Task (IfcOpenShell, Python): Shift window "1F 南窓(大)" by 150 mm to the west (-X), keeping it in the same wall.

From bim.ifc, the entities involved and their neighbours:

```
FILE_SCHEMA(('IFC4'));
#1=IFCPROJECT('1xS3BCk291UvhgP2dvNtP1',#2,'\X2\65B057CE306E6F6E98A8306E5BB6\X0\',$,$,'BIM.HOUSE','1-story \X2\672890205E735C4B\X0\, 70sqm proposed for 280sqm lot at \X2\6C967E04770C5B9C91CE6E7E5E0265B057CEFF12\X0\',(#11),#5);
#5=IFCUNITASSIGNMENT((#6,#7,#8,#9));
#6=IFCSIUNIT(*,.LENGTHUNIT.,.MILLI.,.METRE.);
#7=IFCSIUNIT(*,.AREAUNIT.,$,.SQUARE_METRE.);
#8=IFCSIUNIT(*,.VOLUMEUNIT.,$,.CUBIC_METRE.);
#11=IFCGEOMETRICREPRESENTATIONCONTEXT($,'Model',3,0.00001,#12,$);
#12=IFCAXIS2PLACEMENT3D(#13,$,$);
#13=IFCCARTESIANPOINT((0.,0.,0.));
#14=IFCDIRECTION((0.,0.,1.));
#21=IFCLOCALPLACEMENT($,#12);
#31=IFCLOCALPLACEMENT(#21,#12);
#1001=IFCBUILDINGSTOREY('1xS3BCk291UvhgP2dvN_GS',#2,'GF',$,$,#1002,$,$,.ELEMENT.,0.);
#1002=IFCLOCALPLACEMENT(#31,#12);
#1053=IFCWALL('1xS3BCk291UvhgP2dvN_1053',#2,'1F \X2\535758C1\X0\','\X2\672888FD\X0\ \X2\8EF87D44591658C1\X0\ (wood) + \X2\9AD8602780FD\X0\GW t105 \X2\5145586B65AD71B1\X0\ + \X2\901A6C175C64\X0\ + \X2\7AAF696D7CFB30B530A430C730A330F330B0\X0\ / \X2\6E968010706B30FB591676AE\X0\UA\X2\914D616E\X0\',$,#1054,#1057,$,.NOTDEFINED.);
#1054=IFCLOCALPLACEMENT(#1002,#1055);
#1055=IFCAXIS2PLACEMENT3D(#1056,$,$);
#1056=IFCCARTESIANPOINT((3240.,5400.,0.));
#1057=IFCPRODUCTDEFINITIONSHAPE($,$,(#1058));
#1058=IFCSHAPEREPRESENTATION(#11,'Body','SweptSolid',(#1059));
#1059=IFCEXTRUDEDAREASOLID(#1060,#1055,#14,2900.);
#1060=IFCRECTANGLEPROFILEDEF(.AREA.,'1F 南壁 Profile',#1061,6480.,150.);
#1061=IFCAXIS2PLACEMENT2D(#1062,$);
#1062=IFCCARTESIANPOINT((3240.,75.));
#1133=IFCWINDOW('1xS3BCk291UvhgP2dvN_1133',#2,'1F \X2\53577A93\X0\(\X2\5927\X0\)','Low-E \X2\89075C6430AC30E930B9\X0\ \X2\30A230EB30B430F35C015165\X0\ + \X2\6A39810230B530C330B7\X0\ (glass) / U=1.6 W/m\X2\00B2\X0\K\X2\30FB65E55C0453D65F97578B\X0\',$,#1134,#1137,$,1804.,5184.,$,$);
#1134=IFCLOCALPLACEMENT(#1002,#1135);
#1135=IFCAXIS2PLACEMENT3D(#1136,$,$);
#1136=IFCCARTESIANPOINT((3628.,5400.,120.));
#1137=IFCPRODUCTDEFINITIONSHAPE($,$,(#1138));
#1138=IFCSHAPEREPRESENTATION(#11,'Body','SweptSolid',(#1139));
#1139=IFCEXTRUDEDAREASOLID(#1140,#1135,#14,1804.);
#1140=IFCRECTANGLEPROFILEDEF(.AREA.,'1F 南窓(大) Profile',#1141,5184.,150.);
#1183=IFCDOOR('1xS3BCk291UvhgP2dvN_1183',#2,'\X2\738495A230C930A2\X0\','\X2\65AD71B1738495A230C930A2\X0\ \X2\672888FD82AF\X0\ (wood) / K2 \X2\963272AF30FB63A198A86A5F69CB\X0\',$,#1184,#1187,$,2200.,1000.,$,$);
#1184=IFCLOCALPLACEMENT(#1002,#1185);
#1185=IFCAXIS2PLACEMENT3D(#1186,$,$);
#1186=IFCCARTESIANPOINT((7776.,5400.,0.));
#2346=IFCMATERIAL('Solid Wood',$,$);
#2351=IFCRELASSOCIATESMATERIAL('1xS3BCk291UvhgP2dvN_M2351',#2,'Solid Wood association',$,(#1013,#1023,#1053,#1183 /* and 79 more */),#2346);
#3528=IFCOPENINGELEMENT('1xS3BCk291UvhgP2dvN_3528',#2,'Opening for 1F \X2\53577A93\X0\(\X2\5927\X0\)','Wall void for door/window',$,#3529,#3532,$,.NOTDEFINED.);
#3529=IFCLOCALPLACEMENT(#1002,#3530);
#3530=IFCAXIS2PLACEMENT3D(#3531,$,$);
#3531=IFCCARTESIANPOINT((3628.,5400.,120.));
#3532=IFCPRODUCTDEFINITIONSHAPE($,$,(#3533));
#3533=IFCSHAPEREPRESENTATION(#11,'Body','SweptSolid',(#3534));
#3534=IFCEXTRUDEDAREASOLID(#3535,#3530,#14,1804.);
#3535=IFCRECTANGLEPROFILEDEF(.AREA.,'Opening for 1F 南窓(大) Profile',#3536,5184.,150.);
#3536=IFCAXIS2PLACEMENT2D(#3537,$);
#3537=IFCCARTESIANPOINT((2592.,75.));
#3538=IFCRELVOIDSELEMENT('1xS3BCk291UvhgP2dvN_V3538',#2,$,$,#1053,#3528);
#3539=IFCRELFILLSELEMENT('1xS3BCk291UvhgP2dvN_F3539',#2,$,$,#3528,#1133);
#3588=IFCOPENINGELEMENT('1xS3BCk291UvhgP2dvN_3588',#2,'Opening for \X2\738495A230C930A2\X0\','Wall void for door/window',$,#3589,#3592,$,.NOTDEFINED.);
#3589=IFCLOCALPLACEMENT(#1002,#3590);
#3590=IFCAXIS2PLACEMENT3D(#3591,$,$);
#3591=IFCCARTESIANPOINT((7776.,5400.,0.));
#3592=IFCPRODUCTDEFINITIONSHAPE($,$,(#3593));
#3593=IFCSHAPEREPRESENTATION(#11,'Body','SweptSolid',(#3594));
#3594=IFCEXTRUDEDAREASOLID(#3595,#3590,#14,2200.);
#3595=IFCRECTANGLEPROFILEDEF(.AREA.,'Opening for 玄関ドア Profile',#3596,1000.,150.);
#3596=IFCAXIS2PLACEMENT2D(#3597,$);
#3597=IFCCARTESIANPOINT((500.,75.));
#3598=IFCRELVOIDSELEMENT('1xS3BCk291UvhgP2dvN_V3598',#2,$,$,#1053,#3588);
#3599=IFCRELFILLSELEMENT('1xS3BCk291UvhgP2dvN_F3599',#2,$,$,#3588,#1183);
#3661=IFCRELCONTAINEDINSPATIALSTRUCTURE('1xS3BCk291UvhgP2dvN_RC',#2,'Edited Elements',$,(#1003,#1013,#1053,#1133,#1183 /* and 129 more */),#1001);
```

```python
import ifcopenshell
import ifcopenshell.api.geometry
import ifcopenshell.util.placement
import ifcopenshell.util.unit

model = ifcopenshell.open("bim.ifc")
unit_scale = ifcopenshell.util.unit.calculate_unit_scale(model)

window = model.by_guid("1xS3BCk291UvhgP2dvN_1133")
opening = window.FillsVoids[0].RelatingOpeningElement
wall = opening.VoidsElements[0].RelatingBuildingElement

wall_matrix = ifcopenshell.util.placement.get_local_placement(wall.ObjectPlacement)
shift = wall_matrix[:3, 0] * -0.15 / unit_scale
before = ifcopenshell.util.placement.get_local_placement(window.ObjectPlacement)[:3, 3].copy()

# The window is not placed relative to its opening, so move both.
for product in (opening, window):
    matrix = ifcopenshell.util.placement.get_local_placement(product.ObjectPlacement)
    matrix[:3, 3] += shift
    ifcopenshell.api.geometry.edit_object_placement(model, product=product, matrix=matrix, is_si=False)

after = ifcopenshell.util.placement.get_local_placement(window.ObjectPlacement)[:3, 3]
print("window moved by", (after - before).round(3) + 0.0)

model.write("bim-out.ifc")
```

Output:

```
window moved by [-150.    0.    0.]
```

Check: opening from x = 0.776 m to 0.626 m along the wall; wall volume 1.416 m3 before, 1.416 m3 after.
